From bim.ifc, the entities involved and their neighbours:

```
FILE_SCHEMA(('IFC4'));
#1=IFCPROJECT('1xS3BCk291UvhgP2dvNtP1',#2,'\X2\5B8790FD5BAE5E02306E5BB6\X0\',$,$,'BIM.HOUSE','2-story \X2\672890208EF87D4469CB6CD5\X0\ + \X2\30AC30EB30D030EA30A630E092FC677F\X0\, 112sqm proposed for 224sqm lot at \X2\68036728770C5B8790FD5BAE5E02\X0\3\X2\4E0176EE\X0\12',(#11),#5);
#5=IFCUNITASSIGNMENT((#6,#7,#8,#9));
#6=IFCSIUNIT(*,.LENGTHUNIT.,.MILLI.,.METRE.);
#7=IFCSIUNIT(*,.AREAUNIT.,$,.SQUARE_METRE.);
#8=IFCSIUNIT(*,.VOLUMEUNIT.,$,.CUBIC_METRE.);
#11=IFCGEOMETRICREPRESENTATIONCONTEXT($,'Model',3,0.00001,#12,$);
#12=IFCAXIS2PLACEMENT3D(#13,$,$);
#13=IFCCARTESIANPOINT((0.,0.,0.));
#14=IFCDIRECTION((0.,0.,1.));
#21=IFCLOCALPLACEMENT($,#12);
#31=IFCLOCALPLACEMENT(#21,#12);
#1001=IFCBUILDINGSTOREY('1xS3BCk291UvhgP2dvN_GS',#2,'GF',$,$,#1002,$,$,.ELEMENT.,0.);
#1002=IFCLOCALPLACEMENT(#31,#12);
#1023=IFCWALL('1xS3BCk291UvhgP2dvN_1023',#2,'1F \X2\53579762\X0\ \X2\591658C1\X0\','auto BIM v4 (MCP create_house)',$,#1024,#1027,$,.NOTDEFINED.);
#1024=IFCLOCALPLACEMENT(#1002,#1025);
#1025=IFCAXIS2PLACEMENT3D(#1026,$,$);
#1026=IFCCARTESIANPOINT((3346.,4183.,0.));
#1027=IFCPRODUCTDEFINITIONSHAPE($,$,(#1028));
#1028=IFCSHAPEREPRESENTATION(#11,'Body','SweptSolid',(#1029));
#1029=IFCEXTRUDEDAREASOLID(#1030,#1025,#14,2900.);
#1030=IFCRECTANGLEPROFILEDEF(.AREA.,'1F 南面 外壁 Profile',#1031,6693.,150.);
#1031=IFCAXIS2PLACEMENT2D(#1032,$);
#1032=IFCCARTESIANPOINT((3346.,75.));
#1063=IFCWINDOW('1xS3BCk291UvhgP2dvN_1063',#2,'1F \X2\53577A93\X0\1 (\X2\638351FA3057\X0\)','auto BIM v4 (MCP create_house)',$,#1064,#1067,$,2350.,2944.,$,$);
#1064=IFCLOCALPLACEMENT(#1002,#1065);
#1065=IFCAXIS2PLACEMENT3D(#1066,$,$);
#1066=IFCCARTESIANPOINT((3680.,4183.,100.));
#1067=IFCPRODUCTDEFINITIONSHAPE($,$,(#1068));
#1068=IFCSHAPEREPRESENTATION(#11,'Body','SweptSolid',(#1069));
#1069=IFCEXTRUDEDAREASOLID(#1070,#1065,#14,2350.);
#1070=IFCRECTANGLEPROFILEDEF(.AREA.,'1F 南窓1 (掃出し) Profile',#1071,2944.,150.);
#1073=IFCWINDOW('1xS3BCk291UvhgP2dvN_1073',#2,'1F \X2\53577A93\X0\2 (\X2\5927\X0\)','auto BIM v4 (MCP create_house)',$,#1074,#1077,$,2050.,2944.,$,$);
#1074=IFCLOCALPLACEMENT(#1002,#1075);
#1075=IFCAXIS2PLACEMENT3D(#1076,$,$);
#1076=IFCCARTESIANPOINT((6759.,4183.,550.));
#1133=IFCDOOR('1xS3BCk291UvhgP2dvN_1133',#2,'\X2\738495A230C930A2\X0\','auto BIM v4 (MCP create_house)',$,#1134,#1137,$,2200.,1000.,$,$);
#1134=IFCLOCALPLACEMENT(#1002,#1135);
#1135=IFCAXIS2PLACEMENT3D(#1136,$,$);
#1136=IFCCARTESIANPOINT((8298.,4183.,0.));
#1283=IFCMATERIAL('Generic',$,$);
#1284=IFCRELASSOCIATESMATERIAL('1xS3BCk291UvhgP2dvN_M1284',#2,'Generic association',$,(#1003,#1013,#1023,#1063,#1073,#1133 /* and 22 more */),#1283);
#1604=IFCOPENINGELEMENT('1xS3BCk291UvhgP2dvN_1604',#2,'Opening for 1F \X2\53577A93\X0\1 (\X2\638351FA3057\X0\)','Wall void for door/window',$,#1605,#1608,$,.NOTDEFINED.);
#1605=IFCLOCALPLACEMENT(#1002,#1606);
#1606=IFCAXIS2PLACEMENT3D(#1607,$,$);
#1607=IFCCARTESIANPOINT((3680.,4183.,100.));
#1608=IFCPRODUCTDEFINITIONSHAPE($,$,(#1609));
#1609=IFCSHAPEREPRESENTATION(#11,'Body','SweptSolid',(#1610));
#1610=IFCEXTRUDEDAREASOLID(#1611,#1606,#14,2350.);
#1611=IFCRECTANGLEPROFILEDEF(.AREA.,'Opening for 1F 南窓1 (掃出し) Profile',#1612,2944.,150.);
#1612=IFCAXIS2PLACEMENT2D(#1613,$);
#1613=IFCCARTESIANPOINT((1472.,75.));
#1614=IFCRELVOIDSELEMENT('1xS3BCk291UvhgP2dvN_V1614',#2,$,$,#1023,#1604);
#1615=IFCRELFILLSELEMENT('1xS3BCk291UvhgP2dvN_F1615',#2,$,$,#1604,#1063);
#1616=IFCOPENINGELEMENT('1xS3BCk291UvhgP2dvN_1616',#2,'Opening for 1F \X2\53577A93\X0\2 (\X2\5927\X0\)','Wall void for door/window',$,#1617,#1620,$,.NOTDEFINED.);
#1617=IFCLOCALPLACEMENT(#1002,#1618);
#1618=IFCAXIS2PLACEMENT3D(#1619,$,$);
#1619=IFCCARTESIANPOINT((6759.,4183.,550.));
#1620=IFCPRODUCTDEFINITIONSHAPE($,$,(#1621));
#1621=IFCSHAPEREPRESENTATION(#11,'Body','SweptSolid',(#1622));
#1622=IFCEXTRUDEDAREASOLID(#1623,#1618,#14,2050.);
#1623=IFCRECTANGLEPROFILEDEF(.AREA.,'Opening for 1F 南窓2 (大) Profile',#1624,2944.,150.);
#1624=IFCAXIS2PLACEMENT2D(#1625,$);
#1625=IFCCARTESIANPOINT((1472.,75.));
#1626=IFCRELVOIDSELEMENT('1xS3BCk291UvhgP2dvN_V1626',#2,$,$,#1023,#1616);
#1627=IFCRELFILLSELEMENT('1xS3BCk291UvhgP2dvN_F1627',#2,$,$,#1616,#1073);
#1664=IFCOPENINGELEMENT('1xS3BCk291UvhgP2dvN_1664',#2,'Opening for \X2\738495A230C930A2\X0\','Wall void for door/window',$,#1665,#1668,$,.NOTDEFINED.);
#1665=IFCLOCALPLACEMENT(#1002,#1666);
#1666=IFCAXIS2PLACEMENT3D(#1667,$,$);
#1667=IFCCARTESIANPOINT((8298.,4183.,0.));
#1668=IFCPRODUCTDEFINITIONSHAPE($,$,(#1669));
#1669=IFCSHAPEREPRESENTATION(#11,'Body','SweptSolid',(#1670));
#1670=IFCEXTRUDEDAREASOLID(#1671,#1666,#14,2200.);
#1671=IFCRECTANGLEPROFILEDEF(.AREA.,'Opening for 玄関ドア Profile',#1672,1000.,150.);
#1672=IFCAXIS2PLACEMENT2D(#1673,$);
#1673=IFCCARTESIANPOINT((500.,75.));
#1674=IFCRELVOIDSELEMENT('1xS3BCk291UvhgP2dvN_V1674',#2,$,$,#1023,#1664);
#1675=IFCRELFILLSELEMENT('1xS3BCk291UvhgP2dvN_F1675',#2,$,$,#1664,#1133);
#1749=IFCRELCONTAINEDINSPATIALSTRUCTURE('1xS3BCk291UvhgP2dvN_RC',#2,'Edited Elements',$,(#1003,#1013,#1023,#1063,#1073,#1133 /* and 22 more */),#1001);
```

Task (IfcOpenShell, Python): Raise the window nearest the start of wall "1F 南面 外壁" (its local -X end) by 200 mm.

```python
import numpy as np
import ifcopenshell
import ifcopenshell.api.geometry
import ifcopenshell.util.placement
import ifcopenshell.util.unit

model = ifcopenshell.open("bim.ifc")
unit_scale = ifcopenshell.util.unit.calculate_unit_scale(model)

window = model.by_id(1063)
opening = window.FillsVoids[0].RelatingOpeningElement
dz = 200.0

shift = np.array([0.0, 0.0, dz])
# The window is not placed relative to its opening, so move both.
for product in (opening, window):
    matrix = ifcopenshell.util.placement.get_local_placement(product.ObjectPlacement)
    matrix[:3, 3] += shift
    ifcopenshell.api.geometry.edit_object_placement(model, product=product, matrix=matrix, is_si=False)

print(f"moved by {dz * unit_scale:+.3f} m")

model.write("bim-out.ifc")
```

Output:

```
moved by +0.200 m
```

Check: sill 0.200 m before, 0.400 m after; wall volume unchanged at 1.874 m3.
